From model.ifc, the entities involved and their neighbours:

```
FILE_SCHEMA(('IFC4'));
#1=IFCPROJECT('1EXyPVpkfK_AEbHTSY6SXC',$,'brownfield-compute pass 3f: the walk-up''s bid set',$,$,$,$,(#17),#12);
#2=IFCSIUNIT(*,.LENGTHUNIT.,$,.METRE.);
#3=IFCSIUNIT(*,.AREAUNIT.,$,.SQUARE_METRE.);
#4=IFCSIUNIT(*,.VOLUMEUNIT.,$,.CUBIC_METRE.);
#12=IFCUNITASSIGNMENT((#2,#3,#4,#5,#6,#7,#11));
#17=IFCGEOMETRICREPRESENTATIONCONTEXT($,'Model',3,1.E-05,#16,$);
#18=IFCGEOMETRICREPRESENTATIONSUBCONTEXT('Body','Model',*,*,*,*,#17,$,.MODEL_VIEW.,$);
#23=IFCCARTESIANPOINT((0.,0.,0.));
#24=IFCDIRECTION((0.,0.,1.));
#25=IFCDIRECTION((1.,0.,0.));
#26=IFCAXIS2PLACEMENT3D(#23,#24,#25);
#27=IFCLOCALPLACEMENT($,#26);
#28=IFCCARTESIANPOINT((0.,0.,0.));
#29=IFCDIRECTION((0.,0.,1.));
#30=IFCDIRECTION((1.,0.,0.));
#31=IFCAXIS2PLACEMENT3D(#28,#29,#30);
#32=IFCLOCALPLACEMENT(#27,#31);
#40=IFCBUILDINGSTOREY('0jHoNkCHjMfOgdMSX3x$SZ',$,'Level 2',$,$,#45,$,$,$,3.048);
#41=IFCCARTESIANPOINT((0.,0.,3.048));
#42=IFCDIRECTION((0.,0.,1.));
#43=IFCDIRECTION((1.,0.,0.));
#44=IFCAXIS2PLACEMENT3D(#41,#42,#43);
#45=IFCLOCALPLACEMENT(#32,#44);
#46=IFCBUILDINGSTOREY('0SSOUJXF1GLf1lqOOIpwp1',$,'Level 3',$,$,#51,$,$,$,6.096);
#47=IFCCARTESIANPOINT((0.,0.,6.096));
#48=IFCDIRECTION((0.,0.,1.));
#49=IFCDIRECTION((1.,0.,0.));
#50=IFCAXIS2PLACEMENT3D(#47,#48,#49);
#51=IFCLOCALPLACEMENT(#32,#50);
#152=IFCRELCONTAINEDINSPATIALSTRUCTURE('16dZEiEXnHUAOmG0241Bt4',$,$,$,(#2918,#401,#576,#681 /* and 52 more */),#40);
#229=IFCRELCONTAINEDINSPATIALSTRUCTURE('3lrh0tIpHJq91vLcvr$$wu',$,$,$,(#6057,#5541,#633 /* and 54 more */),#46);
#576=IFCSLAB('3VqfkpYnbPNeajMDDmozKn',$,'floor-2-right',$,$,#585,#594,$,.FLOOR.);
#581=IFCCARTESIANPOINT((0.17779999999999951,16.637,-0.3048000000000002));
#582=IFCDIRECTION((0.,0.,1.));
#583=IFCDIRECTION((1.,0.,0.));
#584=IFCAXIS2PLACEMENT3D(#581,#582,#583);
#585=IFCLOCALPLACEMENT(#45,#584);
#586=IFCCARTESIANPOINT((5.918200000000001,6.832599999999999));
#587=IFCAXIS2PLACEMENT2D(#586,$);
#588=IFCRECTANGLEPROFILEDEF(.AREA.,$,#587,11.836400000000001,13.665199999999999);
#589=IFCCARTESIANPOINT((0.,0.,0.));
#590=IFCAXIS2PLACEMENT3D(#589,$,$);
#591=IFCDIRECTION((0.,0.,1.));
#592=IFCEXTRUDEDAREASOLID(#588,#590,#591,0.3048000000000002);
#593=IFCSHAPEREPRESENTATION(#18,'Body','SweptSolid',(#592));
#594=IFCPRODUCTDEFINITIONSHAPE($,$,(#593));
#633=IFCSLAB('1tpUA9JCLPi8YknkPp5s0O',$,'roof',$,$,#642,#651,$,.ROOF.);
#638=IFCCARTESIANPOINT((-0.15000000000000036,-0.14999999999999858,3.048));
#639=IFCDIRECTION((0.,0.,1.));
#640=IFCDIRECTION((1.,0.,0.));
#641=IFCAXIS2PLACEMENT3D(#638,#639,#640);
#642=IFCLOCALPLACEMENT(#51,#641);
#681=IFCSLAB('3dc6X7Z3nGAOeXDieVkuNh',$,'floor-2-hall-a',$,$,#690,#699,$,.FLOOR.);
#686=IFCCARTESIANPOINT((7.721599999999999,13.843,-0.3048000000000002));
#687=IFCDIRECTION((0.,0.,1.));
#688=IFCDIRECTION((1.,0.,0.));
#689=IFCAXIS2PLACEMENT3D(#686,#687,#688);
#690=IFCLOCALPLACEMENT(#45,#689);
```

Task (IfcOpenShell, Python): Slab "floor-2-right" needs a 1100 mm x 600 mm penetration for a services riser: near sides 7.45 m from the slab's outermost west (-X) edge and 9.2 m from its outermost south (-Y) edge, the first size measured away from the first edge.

```python
import numpy as np
import ifcopenshell
import ifcopenshell.api.feature
import ifcopenshell.api.geometry
import ifcopenshell.api.root
import ifcopenshell.geom
import ifcopenshell.util.placement
import ifcopenshell.util.representation
import ifcopenshell.util.shape
import ifcopenshell.util.unit

model = ifcopenshell.open("model.ifc")
unit_scale = ifcopenshell.util.unit.calculate_unit_scale(model)
settings = ifcopenshell.geom.settings()


def volume(element):
    """Net volume in cubic metres, openings subtracted."""
    shape = ifcopenshell.geom.create_shape(settings, element)
    return ifcopenshell.util.shape.get_volume(shape.geometry)


slab = model.by_guid("3VqfkpYnbPNeajMDDmozKn")
before = volume(slab)

# Extent in the slab's own axes, in metres. The edges named are its -X and -Y sides.
slab_shape = ifcopenshell.geom.create_shape(settings, slab)
vertices = ifcopenshell.util.shape.get_vertices(slab_shape.geometry)
x_min, y_min, bottom = vertices.min(axis=0)
top = vertices[:, 2].max()

opening = ifcopenshell.api.root.create_entity(model, ifc_class="IfcOpeningElement", name="Services riser opening", predefined_type="OPENING")
context = ifcopenshell.util.representation.get_context(model, "Model", "Body", "MODEL_VIEW")
width, depth = 1.1, 0.6
outline = [(0.0, 0.0), (width, 0.0), (width, depth), (0.0, depth), (0.0, 0.0)]
# Overshoot both faces by 50 mm so the cut is clean.
shape = ifcopenshell.api.geometry.add_slab_representation(
    model, context=context, depth=top - bottom + 0.1, polyline=outline
)
ifcopenshell.api.geometry.assign_representation(model, product=opening, representation=shape)

matrix = ifcopenshell.util.placement.get_local_placement(slab.ObjectPlacement)
matrix[:, 3] = matrix @ np.append(np.array([x_min + 7.45, y_min + 9.2, bottom - 0.05]) / unit_scale, 1.0)
ifcopenshell.api.geometry.edit_object_placement(model, product=opening, matrix=matrix, is_si=False)
ifcopenshell.api.feature.add_feature(model, feature=opening, element=slab)

after = volume(slab)

print(f"slab volume {before:.3f} -> {after:.3f} m3")

model.write("model_edited.ifc")
```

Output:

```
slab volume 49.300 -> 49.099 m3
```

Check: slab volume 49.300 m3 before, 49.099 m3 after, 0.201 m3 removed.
